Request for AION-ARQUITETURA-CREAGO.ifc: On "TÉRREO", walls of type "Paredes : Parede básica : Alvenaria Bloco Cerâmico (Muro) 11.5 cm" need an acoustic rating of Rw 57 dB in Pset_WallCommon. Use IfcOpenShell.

First a look at what the model holds.

```python
import ifcopenshell
import ifcopenshell.util.element

model = ifcopenshell.open("AION-ARQUITETURA-CREAGO.ifc")
print(model.schema)
storey = next(s for s in model.by_type("IfcBuildingStorey") if s.Name == "TÉRREO")
walls = [e for e in ifcopenshell.util.element.get_decomposition(storey) if e.is_a("IfcWall")]
seen = {}
for e in walls:
    element_type = ifcopenshell.util.element.get_type(e)
    key = (element_type.Name if element_type != e and element_type else None, ifcopenshell.util.element.get_pset(e, "Pset_WallCommon", "AcousticRating"))
    seen[key] = seen.get(key, 0) + 1
for (name, value), count in sorted(seen.items(), key=str):
    print(count, "x", name, "|", value)
```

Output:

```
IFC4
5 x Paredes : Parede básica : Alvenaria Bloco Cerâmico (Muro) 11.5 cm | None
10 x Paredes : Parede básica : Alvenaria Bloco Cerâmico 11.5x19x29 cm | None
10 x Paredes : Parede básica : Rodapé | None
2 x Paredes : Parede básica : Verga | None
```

```python
import ifcopenshell
import ifcopenshell.api.pset
import ifcopenshell.util.element

model = ifcopenshell.open("AION-ARQUITETURA-CREAGO.ifc")

storey = next(s for s in model.by_type("IfcBuildingStorey") if s.Name == "TÉRREO")
walls = [e for e in ifcopenshell.util.element.get_decomposition(storey) if e.is_a("IfcWall")]

count = 0
for e in walls:
    element_type = ifcopenshell.util.element.get_type(e)
    if element_type in (None, e) or element_type.Name != "Paredes : Parede básica : Alvenaria Bloco Cerâmico (Muro) 11.5 cm":
        continue
    # add_pset returns the element's existing set when there is one.
    pset = ifcopenshell.api.pset.add_pset(model, product=e, name="Pset_WallCommon")
    ifcopenshell.api.pset.edit_pset(model, pset=pset, properties={"AcousticRating": "Rw 57 dB"})
    count += 1

print(count, "walls updated")

model.write("AION-ARQUITETURA-CREAGO-out.ifc")
```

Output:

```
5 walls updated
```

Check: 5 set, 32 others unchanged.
